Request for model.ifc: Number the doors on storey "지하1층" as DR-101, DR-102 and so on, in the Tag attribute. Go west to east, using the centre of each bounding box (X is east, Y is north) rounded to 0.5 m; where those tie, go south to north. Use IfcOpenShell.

First a look at what the model holds.

```python
import ifcopenshell
import ifcopenshell.util.element
import ifcopenshell.util.placement

model = ifcopenshell.open("model.ifc")
print(model.schema)
storey = next(s for s in model.by_type("IfcBuildingStorey") if s.Name == "지하1층")
doors = [e for e in ifcopenshell.util.element.get_decomposition(storey) if e.is_a("IfcDoor")]
for e in sorted(doors, key=lambda e: e.id()):
    origin = ifcopenshell.util.placement.get_local_placement(e.ObjectPlacement)[:3, 3]
    print(e.id(), e.Tag, e.Name, origin.round(2) + 0.0, sep=" | ")
```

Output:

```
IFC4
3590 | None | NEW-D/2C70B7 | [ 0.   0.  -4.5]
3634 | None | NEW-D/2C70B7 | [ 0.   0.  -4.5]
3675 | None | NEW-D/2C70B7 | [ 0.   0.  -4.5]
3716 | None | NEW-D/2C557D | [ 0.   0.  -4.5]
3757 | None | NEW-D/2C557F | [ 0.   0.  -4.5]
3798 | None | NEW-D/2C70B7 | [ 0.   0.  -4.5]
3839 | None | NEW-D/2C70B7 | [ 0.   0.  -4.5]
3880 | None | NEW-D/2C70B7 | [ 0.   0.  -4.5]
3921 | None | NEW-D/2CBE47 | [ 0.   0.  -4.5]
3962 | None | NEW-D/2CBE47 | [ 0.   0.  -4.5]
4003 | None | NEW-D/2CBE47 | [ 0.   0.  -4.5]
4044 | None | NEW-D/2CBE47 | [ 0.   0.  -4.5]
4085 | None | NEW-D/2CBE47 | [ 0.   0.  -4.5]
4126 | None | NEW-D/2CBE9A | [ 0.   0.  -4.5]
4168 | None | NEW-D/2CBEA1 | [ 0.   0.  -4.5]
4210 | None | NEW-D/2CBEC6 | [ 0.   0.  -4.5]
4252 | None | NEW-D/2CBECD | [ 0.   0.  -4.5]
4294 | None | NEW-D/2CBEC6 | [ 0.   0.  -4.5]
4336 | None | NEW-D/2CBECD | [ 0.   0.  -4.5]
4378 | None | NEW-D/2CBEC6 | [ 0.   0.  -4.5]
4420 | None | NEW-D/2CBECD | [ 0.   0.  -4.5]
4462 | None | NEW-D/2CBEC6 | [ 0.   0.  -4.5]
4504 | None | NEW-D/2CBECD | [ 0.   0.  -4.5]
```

```python
import ifcopenshell
import ifcopenshell.geom
import ifcopenshell.util.element
import ifcopenshell.util.shape

model = ifcopenshell.open("model.ifc")
settings = ifcopenshell.geom.settings()
settings.set("use-world-coords", True)


def centre(element):
    shape = ifcopenshell.geom.create_shape(settings, element)
    return ifcopenshell.util.shape.get_bbox_centroid(shape.geometry)


storey = next(s for s in model.by_type("IfcBuildingStorey") if s.Name == "지하1층")
doors = [e for e in ifcopenshell.util.element.get_decomposition(storey) if e.is_a("IfcDoor")]

# Insertion points can sit at a corner or the storey origin, so sort by the geometry (in metres).
centres = {e: centre(e) for e in doors}
doors.sort(key=lambda e: (round(centres[e][0] / 0.5), centres[e][1]))

for i, e in enumerate(doors, start=1):
    number = f"DR-1{i:02d}"
    e.Tag = number
    print(e.id(), number)

model.write("model_edited.ifc")
```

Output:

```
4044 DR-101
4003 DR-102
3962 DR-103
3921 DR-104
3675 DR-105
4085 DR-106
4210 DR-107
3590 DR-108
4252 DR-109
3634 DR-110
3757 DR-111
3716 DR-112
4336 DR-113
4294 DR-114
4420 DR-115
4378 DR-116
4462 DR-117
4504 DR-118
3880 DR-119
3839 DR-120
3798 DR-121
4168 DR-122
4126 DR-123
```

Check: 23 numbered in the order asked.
